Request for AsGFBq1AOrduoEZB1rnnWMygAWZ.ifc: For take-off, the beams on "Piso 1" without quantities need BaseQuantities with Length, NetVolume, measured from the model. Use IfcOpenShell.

First a look at what the model holds.

```python
import ifcopenshell
import ifcopenshell.util.element
import ifcopenshell.util.unit

model = ifcopenshell.open("AsGFBq1AOrduoEZB1rnnWMygAWZ.ifc")
print(model.schema)
for unit_type in ("LENGTHUNIT", "AREAUNIT", "VOLUMEUNIT"):
    print(unit_type, ifcopenshell.util.unit.calculate_unit_scale(model, unit_type))
storey = next(s for s in model.by_type("IfcBuildingStorey") if s.Name == "Piso 1")
beams = [e for e in ifcopenshell.util.element.get_decomposition(storey) if e.is_a("IfcBeam")]
for e in sorted(beams, key=lambda e: e.id()):
    print(e.id(), e.is_a(), e.Name, list(ifcopenshell.util.element.get_psets(e, qtos_only=True)), sep=" | ")
```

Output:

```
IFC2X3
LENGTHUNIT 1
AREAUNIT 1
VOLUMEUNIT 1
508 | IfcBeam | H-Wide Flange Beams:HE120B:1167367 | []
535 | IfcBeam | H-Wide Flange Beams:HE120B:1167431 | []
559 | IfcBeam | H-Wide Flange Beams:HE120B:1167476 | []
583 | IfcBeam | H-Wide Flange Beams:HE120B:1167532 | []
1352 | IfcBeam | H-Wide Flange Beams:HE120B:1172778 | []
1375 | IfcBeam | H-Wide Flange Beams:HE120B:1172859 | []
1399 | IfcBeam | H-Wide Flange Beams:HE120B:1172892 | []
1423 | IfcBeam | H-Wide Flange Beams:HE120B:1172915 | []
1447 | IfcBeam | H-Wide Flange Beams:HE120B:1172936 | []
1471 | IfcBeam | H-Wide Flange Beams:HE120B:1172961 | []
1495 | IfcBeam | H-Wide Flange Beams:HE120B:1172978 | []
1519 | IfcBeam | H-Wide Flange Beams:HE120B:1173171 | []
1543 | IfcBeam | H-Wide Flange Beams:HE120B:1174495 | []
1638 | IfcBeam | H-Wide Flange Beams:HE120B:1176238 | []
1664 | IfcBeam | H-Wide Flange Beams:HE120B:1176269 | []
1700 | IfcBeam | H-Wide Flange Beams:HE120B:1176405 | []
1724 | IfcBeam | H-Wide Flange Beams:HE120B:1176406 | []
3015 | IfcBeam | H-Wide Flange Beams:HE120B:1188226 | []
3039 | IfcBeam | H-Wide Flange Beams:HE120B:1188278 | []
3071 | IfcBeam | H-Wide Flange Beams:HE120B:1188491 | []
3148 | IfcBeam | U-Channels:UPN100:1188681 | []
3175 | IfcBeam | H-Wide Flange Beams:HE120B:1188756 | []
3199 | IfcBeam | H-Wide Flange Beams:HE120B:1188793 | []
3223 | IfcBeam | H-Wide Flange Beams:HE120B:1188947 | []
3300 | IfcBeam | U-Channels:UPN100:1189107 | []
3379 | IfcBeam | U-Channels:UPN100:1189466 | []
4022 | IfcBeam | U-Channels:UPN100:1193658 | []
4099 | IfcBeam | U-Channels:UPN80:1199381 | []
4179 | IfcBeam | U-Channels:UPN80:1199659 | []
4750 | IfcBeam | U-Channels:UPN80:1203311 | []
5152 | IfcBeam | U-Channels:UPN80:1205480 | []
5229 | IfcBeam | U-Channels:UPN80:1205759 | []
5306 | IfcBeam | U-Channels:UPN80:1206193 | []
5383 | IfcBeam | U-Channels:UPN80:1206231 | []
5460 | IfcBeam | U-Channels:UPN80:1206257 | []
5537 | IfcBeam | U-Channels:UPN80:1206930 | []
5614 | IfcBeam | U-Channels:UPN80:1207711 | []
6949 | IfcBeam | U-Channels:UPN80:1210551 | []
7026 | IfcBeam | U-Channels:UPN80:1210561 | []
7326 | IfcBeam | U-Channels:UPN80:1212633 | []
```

```python
import ifcopenshell
import ifcopenshell.api.pset
import ifcopenshell.geom
import ifcopenshell.util.element
import ifcopenshell.util.shape
import ifcopenshell.util.unit

model = ifcopenshell.open("AsGFBq1AOrduoEZB1rnnWMygAWZ.ifc")
unit_scale = ifcopenshell.util.unit.calculate_unit_scale(model)
volume_scale = ifcopenshell.util.unit.calculate_unit_scale(model, "VOLUMEUNIT")
settings = ifcopenshell.geom.settings()

storey = next(s for s in model.by_type("IfcBuildingStorey") if s.Name == "Piso 1")
beams = [e for e in ifcopenshell.util.element.get_decomposition(storey) if e.is_a("IfcBeam")]

for e in sorted(beams, key=lambda e: e.id()):
    if ifcopenshell.util.element.get_psets(e, qtos_only=True, should_inherit=False):
        continue
    # Geometry comes back in metres, in the element's own axes.
    shape = ifcopenshell.geom.create_shape(settings, e)
    values = {
        "Length": ifcopenshell.util.shape.get_max_xyz(shape.geometry) / unit_scale,
        "NetVolume": ifcopenshell.util.shape.get_volume(shape.geometry) / volume_scale,
    }
    qto = ifcopenshell.api.pset.add_qto(model, product=e, name="BaseQuantities")
    ifcopenshell.api.pset.edit_qto(model, qto=qto, properties=values)
    print(e.id(), {k: round(v, 3) for k, v in values.items()})

model.write("AsGFBq1AOrduoEZB1rnnWMygAWZ-out.ifc")
```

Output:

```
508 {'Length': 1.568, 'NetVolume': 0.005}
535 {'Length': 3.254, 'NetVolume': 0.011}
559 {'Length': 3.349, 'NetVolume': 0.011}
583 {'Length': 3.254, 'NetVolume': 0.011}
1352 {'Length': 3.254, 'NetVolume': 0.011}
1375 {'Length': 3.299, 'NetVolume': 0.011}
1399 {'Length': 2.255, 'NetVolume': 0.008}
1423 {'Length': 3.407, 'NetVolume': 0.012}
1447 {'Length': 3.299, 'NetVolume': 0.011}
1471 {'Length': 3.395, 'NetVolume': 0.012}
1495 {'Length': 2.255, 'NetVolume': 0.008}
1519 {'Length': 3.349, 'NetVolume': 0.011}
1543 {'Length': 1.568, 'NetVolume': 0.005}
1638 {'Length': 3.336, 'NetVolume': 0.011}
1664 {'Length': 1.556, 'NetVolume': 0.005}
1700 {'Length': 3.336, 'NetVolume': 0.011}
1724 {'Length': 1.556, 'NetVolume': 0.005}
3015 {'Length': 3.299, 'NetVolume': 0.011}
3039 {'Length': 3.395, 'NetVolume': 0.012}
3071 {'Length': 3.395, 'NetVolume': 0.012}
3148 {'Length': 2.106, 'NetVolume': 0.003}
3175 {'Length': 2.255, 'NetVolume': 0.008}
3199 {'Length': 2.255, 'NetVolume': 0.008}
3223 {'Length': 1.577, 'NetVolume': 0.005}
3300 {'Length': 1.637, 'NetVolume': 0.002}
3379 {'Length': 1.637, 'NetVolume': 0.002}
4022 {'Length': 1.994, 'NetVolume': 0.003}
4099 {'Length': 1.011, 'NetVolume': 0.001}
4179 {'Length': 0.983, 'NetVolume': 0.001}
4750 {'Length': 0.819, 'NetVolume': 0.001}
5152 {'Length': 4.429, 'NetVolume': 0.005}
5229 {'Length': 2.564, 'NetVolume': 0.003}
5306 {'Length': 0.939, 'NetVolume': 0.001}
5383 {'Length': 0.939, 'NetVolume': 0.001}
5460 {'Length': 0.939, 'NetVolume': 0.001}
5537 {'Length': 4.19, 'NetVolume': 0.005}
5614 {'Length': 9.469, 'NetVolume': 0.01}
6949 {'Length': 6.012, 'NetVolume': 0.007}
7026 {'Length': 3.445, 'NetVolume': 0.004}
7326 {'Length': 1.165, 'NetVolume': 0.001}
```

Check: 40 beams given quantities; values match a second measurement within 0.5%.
